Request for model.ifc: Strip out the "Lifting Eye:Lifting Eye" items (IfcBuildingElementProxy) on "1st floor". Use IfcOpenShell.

First a look at what the model holds.

```python
import ifcopenshell
import ifcopenshell.util.element

model = ifcopenshell.open("model.ifc")
print(model.schema)
storey = next(s for s in model.by_type("IfcBuildingStorey") if s.Name == "1st floor")
proxies = [e for e in ifcopenshell.util.element.get_decomposition(storey) if e.is_a("IfcBuildingElementProxy")]
seen = {}
for e in proxies:
    element_type = ifcopenshell.util.element.get_type(e)
    name = element_type.Name if element_type not in (None, e) else None
    seen[name] = seen.get(name, 0) + 1
for name, count in sorted(seen.items(), key=str):
    print(count, "x", name)
```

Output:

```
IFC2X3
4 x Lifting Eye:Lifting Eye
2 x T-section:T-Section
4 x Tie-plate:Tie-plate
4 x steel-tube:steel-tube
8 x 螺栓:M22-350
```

```python
import ifcopenshell
import ifcopenshell.api.root
import ifcopenshell.util.element

model = ifcopenshell.open("model.ifc")

storey = next(s for s in model.by_type("IfcBuildingStorey") if s.Name == "1st floor")
proxies = [e for e in ifcopenshell.util.element.get_decomposition(storey) if e.is_a("IfcBuildingElementProxy")]
targets = [e for e in proxies if (t := ifcopenshell.util.element.get_type(e)) not in (None, e) and t.Name == "Lifting Eye:Lifting Eye"]

for e in targets:
    ifcopenshell.api.root.remove_product(model, product=e)
print(len(targets), "removed")

model.write("model_updated.ifc")
```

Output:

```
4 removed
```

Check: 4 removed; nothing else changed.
